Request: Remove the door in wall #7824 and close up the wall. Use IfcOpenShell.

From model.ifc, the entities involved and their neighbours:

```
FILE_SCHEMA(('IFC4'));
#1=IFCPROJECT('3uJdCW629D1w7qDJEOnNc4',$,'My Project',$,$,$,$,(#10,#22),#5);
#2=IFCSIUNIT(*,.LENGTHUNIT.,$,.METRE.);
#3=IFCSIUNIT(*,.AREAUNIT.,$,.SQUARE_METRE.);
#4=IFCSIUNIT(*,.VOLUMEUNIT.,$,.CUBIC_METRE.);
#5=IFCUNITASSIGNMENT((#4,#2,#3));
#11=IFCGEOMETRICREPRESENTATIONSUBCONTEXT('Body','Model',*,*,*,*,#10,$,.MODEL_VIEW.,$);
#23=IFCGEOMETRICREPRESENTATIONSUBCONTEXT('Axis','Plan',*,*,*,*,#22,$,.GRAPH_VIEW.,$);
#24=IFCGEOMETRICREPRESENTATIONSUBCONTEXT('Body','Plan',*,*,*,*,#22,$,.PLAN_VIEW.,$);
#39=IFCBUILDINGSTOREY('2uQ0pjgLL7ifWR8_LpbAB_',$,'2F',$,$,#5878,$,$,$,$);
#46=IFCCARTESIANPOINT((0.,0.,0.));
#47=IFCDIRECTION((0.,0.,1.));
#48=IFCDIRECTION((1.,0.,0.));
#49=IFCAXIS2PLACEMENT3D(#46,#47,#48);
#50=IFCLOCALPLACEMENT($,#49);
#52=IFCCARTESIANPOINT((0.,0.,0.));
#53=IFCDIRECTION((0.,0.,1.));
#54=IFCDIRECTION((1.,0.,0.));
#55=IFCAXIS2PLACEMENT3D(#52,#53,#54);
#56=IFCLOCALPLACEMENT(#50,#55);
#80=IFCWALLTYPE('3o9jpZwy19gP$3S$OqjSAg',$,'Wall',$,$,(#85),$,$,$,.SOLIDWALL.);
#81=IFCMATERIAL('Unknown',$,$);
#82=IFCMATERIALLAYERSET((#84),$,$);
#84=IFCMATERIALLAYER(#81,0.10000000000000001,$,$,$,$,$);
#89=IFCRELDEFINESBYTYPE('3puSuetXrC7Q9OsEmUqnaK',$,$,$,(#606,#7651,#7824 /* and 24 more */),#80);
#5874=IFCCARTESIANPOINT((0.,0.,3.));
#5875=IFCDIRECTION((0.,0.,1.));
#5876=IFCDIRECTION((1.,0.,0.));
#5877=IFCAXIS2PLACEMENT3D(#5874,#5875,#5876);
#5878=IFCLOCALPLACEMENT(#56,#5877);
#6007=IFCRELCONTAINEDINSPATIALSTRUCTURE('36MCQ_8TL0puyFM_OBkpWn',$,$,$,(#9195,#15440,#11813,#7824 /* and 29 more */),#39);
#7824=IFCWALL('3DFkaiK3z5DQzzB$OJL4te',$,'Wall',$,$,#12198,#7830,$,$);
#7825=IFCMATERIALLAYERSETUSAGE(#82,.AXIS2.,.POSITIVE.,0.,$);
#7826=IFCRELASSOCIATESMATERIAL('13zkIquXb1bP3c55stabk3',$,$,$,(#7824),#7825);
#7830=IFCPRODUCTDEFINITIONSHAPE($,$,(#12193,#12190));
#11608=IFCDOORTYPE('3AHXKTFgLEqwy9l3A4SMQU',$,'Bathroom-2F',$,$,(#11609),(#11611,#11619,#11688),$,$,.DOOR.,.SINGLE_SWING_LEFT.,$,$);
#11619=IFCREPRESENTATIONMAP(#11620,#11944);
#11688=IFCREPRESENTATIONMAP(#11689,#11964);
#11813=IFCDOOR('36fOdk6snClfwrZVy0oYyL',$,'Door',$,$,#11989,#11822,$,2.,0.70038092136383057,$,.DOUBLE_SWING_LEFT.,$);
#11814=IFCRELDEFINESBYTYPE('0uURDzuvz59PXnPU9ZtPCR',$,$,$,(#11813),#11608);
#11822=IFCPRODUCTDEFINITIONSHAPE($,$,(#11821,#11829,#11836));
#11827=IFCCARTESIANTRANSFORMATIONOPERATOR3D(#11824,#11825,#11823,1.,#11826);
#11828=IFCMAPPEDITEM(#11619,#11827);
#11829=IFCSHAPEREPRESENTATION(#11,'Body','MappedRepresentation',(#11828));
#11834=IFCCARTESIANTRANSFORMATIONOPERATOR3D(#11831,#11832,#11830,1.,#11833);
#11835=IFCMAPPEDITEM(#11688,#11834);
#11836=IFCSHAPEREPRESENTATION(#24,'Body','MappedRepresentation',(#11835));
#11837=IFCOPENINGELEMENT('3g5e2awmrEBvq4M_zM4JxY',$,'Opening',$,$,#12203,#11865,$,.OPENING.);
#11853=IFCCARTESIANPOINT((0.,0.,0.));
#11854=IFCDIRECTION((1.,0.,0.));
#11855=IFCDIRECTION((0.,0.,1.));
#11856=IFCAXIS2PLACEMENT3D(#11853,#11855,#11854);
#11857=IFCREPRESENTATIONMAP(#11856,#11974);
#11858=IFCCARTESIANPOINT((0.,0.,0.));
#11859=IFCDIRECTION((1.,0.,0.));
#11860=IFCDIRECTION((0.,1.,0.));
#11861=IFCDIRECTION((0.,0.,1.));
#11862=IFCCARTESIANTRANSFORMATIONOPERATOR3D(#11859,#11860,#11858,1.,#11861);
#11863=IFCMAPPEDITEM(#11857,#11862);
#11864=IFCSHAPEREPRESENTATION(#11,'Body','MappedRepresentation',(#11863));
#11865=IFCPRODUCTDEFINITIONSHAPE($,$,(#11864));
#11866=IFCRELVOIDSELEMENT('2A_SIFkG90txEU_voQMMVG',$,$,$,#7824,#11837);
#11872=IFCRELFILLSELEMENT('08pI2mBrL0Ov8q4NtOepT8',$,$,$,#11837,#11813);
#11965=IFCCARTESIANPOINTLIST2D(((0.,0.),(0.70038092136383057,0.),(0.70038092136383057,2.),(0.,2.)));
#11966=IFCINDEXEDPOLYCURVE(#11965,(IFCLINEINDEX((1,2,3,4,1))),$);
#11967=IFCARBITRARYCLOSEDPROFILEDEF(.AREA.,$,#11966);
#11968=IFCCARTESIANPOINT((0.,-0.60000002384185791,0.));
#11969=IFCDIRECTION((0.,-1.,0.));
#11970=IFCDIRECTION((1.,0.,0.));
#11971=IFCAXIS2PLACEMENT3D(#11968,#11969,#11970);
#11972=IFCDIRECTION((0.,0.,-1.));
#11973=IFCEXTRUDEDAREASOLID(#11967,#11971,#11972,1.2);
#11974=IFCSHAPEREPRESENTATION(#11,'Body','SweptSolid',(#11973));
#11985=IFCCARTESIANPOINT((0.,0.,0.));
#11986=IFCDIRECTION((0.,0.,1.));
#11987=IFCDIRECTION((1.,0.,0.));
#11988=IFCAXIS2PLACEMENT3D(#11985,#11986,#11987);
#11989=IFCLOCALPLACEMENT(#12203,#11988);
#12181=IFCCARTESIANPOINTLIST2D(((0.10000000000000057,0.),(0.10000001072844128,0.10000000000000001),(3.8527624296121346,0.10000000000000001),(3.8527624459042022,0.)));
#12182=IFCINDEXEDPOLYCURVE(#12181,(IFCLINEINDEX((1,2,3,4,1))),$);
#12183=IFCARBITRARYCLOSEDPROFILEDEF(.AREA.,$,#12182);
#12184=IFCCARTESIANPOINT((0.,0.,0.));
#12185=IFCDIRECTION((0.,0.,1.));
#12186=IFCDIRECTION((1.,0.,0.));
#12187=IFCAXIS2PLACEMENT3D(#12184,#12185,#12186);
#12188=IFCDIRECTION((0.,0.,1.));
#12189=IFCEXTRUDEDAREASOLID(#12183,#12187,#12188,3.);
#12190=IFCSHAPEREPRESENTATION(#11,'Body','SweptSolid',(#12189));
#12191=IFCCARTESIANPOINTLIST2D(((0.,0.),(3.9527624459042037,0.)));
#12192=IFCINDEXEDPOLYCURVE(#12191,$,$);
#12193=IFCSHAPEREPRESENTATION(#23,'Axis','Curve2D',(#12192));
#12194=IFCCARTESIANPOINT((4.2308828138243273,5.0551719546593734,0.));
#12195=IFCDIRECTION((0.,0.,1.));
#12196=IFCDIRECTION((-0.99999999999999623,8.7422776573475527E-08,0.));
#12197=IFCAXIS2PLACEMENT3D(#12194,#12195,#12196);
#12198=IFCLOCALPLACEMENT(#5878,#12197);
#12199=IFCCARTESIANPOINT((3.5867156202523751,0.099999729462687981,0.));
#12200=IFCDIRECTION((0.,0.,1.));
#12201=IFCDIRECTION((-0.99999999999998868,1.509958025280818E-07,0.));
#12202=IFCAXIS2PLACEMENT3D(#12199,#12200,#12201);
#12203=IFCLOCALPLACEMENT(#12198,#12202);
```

```python
import ifcopenshell
import ifcopenshell.api.feature
import ifcopenshell.api.root
import ifcopenshell.geom
import ifcopenshell.util.shape

model = ifcopenshell.open("model.ifc")
settings = ifcopenshell.geom.settings()


def volume(element):
    """Net volume in cubic metres, openings subtracted."""
    shape = ifcopenshell.geom.create_shape(settings, element)
    return ifcopenshell.util.shape.get_volume(shape.geometry)


door = model.by_guid("36fOdk6snClfwrZVy0oYyL")
opening = door.FillsVoids[0].RelatingOpeningElement
wall = opening.VoidsElements[0].RelatingBuildingElement
before = volume(wall)

ifcopenshell.api.root.remove_product(model, product=door)
ifcopenshell.api.feature.remove_feature(model, feature=opening)

after = volume(wall)

print(f"wall volume {before:.3f} -> {after:.3f} m3")

model.write("model_edited.ifc")
```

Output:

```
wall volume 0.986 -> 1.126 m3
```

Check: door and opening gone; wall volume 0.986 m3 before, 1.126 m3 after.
